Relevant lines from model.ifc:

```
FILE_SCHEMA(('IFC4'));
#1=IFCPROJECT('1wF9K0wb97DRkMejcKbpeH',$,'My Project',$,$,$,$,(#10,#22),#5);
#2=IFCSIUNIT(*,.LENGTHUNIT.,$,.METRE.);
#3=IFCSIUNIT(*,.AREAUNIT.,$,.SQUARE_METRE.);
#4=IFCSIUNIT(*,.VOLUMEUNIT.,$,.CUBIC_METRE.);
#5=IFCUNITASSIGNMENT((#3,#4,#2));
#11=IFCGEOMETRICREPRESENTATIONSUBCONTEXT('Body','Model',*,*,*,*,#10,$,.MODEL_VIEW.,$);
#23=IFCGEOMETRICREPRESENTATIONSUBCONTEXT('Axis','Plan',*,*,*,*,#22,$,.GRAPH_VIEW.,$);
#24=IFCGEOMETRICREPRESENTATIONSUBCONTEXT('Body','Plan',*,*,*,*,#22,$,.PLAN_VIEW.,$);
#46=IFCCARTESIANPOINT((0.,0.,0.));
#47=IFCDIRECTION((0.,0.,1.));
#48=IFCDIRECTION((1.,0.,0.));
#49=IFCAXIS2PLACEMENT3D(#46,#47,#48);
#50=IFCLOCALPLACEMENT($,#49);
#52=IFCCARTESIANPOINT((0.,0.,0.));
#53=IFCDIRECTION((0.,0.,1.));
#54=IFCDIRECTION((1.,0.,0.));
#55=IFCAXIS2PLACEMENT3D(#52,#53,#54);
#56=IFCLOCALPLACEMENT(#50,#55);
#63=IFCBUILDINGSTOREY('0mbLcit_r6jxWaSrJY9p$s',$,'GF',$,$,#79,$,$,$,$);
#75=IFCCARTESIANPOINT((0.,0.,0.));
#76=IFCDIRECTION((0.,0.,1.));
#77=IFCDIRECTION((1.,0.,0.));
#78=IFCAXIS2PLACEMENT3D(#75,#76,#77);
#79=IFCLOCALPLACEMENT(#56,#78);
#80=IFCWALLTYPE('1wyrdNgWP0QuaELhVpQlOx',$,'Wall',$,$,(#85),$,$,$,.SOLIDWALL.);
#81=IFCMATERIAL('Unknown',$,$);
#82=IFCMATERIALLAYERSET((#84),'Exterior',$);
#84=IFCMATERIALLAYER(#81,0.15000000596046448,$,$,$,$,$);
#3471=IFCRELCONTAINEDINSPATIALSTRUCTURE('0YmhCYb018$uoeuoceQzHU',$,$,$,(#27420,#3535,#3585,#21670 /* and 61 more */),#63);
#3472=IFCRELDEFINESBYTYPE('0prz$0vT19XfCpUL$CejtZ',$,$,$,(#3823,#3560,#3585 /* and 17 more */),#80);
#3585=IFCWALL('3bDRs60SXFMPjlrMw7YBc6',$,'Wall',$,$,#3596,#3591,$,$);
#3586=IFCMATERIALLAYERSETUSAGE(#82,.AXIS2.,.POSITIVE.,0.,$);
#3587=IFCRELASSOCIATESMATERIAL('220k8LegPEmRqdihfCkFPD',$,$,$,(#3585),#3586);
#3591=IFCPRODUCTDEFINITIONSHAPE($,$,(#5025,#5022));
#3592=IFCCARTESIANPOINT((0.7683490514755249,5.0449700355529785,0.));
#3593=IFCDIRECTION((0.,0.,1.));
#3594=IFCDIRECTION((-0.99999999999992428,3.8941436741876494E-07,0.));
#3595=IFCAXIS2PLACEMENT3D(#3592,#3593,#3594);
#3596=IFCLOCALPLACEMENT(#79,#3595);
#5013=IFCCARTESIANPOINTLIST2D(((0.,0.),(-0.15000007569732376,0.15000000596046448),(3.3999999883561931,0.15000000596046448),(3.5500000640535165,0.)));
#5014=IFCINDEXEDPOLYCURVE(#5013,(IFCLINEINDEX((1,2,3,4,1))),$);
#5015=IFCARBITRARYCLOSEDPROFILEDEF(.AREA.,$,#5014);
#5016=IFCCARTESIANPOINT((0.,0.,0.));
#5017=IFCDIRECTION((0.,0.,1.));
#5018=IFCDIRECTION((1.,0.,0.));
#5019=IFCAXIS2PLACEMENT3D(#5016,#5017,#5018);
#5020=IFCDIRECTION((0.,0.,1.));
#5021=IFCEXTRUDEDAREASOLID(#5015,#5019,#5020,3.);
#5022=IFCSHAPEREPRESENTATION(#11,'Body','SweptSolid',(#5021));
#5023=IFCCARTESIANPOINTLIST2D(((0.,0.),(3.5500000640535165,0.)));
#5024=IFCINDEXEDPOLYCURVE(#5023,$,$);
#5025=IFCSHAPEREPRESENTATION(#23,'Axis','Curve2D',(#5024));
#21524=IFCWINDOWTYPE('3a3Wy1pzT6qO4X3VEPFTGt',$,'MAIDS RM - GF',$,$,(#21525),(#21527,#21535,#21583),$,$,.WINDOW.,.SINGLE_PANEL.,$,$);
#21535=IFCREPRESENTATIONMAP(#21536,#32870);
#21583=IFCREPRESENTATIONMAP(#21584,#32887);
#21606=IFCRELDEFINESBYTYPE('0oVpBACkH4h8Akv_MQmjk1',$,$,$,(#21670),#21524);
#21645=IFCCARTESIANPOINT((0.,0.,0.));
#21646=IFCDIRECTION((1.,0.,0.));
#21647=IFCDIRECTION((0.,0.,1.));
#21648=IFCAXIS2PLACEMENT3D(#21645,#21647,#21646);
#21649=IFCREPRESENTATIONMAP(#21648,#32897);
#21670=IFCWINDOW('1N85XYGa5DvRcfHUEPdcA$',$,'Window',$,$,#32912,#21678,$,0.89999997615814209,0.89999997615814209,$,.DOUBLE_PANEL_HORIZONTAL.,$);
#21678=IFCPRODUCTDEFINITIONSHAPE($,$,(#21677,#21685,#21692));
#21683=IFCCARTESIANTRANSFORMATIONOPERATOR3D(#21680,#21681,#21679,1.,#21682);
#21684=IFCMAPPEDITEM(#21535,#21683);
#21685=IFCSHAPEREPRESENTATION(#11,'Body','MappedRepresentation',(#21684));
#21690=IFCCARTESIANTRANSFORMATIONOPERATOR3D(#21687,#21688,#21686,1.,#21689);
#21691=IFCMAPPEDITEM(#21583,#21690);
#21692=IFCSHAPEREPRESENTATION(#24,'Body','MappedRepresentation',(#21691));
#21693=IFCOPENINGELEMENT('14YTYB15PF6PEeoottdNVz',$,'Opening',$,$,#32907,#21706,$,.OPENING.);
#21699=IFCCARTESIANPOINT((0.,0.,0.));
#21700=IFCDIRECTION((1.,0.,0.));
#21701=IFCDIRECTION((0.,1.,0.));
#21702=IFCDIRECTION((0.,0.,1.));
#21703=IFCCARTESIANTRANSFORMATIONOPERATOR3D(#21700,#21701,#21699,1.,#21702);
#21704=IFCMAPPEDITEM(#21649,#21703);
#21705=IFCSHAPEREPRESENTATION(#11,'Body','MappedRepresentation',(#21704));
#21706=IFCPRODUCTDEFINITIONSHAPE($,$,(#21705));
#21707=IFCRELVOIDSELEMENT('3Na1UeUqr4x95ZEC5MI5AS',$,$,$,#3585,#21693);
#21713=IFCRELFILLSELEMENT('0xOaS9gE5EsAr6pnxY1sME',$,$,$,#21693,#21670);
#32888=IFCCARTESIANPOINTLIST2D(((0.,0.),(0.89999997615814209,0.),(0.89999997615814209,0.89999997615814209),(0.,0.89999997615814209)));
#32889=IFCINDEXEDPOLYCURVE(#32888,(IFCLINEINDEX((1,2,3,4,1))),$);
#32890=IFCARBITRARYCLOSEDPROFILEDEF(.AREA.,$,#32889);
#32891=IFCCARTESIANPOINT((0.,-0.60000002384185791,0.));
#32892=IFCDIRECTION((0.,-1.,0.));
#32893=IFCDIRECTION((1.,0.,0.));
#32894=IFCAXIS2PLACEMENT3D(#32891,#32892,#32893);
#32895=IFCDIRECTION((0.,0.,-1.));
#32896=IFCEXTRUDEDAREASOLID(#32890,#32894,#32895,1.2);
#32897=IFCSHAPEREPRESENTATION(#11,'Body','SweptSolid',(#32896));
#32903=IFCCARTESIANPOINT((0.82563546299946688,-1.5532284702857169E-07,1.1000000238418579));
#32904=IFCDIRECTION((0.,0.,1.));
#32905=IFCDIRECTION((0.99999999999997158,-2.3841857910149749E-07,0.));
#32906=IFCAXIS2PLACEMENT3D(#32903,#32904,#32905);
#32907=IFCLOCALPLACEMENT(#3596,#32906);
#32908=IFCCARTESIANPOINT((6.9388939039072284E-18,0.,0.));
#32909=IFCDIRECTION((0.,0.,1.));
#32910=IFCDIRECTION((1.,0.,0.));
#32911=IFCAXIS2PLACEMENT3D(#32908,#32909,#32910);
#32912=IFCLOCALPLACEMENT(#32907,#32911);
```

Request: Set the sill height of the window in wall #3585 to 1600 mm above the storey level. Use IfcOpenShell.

```python
import numpy as np
import ifcopenshell
import ifcopenshell.api.geometry
import ifcopenshell.geom
import ifcopenshell.util.element
import ifcopenshell.util.placement
import ifcopenshell.util.shape
import ifcopenshell.util.unit

model = ifcopenshell.open("model.ifc")
unit_scale = ifcopenshell.util.unit.calculate_unit_scale(model)

window = model.by_id(21670)
opening = window.FillsVoids[0].RelatingOpeningElement
storey = ifcopenshell.util.element.get_container(window, ifc_class="IfcBuildingStorey")
level = ifcopenshell.util.placement.get_local_placement(storey.ObjectPlacement)[2, 3]

# The opening's origin need not be at the sill, so measure its lowest point.
shape = ifcopenshell.geom.create_shape(ifcopenshell.geom.settings(), opening)
bottom = ifcopenshell.util.shape.get_shape_bottom_elevation(shape, shape.geometry) / unit_scale
dz = level + 1.6 - bottom

shift = np.array([0.0, 0.0, dz])
# The window is placed relative to its opening, so it follows when the opening moves.
matrix = ifcopenshell.util.placement.get_local_placement(opening.ObjectPlacement)
matrix[:3, 3] += shift
ifcopenshell.api.geometry.edit_object_placement(
    model, product=opening, matrix=matrix, is_si=False, should_transform_children=True
)

print(f"moved by {dz * unit_scale:+.3f} m")

model.write("model_edited.ifc")
```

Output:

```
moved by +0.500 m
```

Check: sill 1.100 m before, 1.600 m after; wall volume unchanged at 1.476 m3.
